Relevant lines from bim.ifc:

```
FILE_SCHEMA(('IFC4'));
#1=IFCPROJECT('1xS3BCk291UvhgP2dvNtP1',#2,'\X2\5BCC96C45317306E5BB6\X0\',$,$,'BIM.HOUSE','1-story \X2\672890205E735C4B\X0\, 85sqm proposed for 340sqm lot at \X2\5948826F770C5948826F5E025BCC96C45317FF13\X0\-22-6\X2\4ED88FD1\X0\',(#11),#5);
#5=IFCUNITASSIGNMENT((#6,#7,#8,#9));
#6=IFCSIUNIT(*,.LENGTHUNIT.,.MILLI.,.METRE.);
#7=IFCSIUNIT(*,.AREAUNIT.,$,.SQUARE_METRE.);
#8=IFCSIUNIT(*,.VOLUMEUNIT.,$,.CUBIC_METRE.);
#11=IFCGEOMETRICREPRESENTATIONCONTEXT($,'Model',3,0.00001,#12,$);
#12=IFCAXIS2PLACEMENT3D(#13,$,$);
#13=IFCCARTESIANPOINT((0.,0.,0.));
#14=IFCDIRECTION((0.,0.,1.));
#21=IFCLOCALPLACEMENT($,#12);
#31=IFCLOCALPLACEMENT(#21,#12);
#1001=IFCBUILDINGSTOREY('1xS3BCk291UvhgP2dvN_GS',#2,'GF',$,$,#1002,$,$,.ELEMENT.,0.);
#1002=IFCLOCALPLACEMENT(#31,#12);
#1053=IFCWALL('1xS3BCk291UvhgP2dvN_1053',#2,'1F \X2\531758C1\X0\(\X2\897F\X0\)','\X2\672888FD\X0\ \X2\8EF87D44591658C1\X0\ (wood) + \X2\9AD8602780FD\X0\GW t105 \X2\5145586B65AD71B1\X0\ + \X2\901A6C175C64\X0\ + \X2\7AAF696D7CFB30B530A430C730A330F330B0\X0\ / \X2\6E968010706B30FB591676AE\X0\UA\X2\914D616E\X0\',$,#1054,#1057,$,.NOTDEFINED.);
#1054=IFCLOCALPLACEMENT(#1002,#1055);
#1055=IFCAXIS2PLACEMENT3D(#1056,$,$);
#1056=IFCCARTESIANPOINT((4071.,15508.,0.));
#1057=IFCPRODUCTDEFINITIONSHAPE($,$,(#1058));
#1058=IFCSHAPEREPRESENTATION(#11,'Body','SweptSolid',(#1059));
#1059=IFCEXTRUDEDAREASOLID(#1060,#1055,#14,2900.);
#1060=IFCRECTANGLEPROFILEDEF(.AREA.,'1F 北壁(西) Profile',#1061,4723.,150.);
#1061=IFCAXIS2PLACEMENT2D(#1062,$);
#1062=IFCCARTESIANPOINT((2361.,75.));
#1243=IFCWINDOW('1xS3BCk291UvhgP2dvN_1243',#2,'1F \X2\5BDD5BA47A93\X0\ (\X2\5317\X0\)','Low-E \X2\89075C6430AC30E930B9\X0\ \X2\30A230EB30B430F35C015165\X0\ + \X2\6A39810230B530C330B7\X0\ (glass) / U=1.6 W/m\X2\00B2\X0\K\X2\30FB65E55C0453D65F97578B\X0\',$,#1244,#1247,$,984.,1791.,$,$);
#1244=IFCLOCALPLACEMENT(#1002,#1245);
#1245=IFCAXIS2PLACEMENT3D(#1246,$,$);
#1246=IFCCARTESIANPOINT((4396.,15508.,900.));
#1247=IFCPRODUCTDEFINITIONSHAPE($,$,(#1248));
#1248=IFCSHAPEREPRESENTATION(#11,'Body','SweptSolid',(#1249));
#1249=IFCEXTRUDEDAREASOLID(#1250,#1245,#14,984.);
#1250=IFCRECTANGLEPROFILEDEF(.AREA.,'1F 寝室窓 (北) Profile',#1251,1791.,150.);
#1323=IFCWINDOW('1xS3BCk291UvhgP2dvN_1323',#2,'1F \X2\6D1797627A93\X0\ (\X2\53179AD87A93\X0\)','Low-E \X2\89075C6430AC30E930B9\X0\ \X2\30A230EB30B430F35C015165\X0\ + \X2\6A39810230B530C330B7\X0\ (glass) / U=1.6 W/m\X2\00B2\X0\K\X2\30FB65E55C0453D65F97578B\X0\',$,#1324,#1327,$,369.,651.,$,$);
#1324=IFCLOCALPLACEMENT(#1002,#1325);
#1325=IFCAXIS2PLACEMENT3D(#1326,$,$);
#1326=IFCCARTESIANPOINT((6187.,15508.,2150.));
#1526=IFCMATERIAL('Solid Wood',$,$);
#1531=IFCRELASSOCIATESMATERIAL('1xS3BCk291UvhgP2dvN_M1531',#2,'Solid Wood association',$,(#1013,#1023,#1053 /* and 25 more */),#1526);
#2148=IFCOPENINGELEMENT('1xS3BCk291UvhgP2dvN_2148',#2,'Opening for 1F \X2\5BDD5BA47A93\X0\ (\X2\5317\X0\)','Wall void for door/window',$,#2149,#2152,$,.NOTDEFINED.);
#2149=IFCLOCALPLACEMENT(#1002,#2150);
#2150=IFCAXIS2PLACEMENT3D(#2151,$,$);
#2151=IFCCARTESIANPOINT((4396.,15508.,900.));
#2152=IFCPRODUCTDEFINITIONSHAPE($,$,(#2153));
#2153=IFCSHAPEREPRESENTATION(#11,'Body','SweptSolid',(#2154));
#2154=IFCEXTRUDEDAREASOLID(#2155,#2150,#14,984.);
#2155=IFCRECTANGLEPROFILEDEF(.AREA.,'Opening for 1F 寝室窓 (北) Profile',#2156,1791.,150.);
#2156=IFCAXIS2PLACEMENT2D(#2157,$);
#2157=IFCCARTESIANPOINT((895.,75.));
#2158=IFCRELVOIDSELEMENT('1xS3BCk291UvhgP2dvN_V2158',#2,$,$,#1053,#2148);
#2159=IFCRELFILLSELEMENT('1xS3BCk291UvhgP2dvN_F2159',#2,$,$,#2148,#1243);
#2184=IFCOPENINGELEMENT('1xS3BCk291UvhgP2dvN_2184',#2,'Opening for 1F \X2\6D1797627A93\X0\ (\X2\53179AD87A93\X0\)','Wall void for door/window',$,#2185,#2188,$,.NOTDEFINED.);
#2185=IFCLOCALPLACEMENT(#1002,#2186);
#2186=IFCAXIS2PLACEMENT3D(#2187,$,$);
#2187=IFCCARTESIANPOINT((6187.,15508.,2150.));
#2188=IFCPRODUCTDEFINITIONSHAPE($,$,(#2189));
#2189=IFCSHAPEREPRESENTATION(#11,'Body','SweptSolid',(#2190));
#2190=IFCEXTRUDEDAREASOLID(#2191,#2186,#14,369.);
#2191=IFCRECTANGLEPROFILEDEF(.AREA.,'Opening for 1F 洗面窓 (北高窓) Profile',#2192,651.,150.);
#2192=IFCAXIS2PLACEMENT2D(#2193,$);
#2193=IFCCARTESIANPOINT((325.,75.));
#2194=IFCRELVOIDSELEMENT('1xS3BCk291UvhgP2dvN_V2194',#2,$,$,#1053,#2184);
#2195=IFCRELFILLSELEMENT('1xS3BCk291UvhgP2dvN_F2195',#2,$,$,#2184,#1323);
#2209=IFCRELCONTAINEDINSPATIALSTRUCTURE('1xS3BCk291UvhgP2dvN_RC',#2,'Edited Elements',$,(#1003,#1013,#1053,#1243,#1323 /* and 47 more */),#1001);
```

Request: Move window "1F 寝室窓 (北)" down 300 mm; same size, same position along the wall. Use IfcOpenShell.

```python
import numpy as np
import ifcopenshell
import ifcopenshell.api.geometry
import ifcopenshell.util.placement
import ifcopenshell.util.unit

model = ifcopenshell.open("bim.ifc")
unit_scale = ifcopenshell.util.unit.calculate_unit_scale(model)

window = model.by_id(1243)
opening = window.FillsVoids[0].RelatingOpeningElement
dz = -0.3 / unit_scale

shift = np.array([0.0, 0.0, dz])
# The window is not placed relative to its opening, so move both.
for product in (opening, window):
    matrix = ifcopenshell.util.placement.get_local_placement(product.ObjectPlacement)
    matrix[:3, 3] += shift
    ifcopenshell.api.geometry.edit_object_placement(model, product=product, matrix=matrix, is_si=False)

print(f"moved by {dz * unit_scale:+.3f} m")

model.write("bim-out.ifc")
```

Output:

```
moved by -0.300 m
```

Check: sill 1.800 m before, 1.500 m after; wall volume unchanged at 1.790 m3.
